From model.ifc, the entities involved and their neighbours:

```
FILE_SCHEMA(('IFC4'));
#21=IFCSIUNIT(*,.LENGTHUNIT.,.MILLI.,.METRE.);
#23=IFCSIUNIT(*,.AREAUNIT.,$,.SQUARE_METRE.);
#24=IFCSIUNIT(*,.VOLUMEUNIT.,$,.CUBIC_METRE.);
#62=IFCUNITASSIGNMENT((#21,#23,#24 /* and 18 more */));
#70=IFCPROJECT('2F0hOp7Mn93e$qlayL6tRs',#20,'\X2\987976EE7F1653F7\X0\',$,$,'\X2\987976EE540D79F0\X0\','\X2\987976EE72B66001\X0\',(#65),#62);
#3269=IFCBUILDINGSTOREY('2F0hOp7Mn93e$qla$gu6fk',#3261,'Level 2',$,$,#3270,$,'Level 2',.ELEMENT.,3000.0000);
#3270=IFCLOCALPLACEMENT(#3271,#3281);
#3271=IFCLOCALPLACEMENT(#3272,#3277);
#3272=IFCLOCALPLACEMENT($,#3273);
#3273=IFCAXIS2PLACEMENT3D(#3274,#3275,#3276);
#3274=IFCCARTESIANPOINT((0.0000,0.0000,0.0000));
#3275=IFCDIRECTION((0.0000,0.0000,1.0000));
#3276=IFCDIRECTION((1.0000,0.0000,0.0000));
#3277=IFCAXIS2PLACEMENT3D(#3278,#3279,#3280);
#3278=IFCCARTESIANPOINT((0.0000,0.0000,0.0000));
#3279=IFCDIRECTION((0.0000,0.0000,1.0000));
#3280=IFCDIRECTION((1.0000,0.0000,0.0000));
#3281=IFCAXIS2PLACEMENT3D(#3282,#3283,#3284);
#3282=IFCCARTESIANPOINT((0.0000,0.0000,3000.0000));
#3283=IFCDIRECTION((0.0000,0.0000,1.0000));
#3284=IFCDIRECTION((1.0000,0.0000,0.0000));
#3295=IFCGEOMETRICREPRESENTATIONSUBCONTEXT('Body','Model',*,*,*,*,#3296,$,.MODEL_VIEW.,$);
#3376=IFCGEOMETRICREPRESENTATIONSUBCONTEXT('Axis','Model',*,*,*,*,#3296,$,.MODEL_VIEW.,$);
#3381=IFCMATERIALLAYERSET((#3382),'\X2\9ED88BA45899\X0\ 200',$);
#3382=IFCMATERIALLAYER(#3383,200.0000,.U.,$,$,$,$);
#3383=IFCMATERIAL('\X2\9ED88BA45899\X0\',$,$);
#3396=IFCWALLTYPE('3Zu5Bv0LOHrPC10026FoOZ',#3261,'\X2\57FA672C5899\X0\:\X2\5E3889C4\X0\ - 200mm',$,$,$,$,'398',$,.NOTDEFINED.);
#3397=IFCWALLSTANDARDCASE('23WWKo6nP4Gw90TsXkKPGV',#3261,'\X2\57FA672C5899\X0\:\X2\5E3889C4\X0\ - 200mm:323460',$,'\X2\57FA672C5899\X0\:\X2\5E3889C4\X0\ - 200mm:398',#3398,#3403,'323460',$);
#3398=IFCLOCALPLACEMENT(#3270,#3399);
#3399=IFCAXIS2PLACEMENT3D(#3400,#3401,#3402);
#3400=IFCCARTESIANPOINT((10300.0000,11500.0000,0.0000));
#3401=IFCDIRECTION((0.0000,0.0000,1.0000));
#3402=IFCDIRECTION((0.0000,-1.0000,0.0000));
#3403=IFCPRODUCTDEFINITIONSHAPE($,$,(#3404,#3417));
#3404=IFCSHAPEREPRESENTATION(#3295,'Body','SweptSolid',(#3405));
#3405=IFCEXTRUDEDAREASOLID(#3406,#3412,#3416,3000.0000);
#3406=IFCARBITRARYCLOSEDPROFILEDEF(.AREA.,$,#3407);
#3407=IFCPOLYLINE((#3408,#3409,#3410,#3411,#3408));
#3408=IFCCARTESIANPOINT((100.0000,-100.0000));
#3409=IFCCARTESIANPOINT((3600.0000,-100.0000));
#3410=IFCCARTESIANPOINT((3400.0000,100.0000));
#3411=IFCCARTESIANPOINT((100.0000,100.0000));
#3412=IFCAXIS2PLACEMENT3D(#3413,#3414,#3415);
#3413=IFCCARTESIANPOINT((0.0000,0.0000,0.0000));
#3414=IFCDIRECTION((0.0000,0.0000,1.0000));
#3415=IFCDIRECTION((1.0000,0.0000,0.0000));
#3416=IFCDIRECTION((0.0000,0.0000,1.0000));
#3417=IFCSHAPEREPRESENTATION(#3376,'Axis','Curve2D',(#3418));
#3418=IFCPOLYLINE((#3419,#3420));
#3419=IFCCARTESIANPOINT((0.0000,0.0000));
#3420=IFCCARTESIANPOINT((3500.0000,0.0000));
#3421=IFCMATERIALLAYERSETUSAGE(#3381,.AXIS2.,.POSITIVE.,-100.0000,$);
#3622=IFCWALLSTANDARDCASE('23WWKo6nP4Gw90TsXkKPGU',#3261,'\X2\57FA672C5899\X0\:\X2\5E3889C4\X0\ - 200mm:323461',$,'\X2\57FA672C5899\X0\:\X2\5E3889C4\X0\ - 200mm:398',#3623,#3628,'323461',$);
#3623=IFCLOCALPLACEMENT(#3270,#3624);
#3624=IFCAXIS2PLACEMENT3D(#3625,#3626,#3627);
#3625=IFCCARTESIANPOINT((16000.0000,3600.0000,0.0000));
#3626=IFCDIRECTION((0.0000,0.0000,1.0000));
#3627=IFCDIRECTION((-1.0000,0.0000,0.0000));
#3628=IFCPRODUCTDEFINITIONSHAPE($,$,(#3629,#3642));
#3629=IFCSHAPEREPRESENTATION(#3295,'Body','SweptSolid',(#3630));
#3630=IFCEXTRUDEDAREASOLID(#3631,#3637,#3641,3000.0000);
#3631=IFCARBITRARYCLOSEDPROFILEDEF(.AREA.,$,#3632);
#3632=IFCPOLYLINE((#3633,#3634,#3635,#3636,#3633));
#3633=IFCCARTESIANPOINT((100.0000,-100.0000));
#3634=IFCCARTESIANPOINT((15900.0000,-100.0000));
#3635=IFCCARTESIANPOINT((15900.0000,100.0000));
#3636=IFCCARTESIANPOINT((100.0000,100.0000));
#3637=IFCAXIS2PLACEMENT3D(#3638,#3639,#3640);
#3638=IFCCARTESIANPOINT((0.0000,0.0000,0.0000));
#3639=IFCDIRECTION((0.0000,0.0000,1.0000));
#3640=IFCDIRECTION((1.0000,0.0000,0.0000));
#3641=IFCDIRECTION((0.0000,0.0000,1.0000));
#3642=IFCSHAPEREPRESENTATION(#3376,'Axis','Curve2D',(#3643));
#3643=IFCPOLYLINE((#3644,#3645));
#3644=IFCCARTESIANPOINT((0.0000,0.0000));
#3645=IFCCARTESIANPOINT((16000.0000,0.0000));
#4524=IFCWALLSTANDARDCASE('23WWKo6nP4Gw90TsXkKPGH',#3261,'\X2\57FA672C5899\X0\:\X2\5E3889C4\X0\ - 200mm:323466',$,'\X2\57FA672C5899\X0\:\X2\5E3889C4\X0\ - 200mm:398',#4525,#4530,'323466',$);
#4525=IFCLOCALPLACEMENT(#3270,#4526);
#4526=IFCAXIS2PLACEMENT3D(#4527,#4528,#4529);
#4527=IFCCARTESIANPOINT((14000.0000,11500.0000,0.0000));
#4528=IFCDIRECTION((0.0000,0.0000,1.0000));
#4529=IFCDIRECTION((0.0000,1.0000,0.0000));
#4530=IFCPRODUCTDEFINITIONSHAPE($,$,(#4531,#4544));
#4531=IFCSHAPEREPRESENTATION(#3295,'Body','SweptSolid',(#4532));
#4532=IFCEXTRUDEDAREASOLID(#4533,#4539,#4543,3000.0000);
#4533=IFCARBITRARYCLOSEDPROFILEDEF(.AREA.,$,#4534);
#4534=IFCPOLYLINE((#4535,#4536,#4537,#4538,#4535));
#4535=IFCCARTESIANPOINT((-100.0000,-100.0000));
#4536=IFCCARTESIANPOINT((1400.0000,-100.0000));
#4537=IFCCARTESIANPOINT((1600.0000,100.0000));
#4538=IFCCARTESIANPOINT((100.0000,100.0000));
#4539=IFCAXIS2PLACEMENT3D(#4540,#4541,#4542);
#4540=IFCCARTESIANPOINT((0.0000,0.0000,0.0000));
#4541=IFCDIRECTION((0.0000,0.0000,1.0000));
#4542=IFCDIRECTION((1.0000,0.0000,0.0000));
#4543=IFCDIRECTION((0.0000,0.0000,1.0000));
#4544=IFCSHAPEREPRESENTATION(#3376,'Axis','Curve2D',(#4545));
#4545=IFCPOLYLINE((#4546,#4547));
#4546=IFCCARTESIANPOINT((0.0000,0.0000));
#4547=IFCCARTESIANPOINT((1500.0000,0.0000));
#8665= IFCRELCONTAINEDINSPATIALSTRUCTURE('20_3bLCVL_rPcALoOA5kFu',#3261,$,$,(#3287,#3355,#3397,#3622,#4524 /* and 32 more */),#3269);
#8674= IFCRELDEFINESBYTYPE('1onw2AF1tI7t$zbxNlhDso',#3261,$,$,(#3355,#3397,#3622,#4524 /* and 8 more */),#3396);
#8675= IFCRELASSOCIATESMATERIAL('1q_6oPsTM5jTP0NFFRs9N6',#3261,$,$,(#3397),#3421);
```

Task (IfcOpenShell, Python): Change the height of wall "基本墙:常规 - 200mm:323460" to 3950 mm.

```python
import ifcopenshell
import ifcopenshell.geom
import ifcopenshell.util.representation
import ifcopenshell.util.shape
import ifcopenshell.util.unit

model = ifcopenshell.open("model.ifc")
unit_scale = ifcopenshell.util.unit.calculate_unit_scale(model)
settings = ifcopenshell.geom.settings()


def volume(element):
    """Net volume in cubic metres, openings subtracted."""
    shape = ifcopenshell.geom.create_shape(settings, element)
    return ifcopenshell.util.shape.get_volume(shape.geometry)


wall = model.by_guid("23WWKo6nP4Gw90TsXkKPGV")
before = volume(wall)

body = ifcopenshell.util.representation.get_representation(wall, "Model", "Body")
solid = body.Items[0]
old_height = solid.Depth
solid.Depth = 3.95 / unit_scale
after = volume(wall)

print(f"height {old_height:g} -> {solid.Depth:g}, volume {before:.3f} -> {after:.3f} m3")

model.write("model-out.ifc")
```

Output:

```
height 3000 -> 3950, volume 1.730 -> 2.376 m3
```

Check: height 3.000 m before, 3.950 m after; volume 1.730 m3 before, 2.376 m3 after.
